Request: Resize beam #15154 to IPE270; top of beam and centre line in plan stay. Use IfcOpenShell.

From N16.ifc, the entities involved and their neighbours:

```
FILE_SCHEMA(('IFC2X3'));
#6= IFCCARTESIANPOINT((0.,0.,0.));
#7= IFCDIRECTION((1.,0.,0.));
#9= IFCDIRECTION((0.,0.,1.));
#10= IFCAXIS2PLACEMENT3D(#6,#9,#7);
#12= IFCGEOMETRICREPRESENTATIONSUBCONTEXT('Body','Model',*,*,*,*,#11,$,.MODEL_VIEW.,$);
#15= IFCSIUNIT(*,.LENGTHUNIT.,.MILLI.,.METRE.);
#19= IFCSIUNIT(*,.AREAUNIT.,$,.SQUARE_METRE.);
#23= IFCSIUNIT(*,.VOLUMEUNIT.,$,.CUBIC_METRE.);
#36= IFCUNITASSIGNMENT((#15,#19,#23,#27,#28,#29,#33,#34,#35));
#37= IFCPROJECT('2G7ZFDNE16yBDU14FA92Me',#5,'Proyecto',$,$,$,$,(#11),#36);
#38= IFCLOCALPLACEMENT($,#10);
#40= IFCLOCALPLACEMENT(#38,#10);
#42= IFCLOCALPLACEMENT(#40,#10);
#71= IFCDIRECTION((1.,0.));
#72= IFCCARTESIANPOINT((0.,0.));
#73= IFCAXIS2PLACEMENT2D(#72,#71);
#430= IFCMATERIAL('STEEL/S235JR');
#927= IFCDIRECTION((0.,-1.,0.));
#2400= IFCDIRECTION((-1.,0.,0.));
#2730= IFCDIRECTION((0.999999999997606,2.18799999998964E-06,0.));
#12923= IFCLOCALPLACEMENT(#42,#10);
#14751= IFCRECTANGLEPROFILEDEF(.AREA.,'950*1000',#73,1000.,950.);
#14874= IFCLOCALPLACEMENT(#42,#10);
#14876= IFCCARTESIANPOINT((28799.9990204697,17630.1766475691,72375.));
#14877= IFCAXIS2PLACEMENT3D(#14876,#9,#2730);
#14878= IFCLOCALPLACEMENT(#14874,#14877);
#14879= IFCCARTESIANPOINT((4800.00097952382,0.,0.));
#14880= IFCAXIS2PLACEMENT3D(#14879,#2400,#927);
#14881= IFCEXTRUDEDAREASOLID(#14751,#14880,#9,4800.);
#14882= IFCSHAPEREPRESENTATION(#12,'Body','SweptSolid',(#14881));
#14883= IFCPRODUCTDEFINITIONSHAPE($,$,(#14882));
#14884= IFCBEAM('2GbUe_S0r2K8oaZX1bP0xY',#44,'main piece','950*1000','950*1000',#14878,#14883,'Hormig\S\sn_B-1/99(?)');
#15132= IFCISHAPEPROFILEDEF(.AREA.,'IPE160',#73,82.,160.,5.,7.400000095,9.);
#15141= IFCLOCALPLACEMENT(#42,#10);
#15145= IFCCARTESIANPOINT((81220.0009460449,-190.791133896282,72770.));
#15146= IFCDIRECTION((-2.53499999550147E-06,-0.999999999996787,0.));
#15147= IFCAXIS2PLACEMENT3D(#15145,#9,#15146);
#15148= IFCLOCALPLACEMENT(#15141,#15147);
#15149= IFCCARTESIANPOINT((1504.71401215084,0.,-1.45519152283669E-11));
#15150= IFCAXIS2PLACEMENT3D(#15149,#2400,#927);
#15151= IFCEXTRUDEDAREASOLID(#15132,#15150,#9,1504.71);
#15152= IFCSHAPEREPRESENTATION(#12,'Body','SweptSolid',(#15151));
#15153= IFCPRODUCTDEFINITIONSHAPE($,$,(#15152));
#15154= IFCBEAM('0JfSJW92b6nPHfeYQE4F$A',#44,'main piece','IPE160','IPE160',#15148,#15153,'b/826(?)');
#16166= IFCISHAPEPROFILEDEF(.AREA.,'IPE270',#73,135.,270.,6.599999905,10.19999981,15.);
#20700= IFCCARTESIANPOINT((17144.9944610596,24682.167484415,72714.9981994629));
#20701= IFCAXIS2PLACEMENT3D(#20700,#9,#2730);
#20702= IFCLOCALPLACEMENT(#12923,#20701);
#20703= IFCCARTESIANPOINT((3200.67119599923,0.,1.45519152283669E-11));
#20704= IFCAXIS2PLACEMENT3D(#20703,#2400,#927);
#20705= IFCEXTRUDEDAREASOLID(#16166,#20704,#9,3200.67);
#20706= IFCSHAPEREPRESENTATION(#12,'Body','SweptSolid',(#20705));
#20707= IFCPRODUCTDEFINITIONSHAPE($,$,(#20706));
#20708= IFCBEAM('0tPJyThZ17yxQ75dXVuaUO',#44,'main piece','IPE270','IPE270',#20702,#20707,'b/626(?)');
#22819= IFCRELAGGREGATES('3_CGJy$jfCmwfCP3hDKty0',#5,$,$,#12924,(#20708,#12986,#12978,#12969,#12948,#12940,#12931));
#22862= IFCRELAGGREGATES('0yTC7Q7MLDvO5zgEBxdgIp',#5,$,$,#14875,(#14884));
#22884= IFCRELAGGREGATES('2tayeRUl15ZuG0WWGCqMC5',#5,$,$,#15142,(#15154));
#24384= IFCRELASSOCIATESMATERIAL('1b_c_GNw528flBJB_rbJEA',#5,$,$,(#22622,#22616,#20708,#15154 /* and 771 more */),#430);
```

```python
import ifcopenshell
import ifcopenshell.util.element
import ifcopenshell.util.representation

model = ifcopenshell.open("N16.ifc")

member = model.by_id(15154)
source = next(p for p in model.by_type("IfcIShapeProfileDef") if p.ProfileName == "IPE270")

body = ifcopenshell.util.representation.get_representation(member, "Model", "Body")
solid = body.Items[0]
old_profile = solid.SweptArea

# Copy the section's sizes but keep this member's own profile position.
profile = ifcopenshell.util.element.copy(model, source)
# Profiles are centred, so shift by half the change in depth to hold the top.
shift = (old_profile.OverallDepth - profile.OverallDepth) / 2
x, y = old_profile.Position.Location.Coordinates
up = (0.0, 1.0)  # upwards, in the solid's own plane
location = model.createIfcCartesianPoint((x + up[0] * shift, y + up[1] * shift))
profile.Position = model.createIfcAxis2Placement2D(location, old_profile.Position.RefDirection)
solid.SweptArea = profile
if not model.get_total_inverses(old_profile):
    ifcopenshell.util.element.remove_deep2(model, old_profile)
member.Description = member.Description.replace("IPE160", "IPE270")
member.ObjectType = member.ObjectType.replace("IPE160", "IPE270")

print(solid.SweptArea)

model.write("N16_v2.ifc")
```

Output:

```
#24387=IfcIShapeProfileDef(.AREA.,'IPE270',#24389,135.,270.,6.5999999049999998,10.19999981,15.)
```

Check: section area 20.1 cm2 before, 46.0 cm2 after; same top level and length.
